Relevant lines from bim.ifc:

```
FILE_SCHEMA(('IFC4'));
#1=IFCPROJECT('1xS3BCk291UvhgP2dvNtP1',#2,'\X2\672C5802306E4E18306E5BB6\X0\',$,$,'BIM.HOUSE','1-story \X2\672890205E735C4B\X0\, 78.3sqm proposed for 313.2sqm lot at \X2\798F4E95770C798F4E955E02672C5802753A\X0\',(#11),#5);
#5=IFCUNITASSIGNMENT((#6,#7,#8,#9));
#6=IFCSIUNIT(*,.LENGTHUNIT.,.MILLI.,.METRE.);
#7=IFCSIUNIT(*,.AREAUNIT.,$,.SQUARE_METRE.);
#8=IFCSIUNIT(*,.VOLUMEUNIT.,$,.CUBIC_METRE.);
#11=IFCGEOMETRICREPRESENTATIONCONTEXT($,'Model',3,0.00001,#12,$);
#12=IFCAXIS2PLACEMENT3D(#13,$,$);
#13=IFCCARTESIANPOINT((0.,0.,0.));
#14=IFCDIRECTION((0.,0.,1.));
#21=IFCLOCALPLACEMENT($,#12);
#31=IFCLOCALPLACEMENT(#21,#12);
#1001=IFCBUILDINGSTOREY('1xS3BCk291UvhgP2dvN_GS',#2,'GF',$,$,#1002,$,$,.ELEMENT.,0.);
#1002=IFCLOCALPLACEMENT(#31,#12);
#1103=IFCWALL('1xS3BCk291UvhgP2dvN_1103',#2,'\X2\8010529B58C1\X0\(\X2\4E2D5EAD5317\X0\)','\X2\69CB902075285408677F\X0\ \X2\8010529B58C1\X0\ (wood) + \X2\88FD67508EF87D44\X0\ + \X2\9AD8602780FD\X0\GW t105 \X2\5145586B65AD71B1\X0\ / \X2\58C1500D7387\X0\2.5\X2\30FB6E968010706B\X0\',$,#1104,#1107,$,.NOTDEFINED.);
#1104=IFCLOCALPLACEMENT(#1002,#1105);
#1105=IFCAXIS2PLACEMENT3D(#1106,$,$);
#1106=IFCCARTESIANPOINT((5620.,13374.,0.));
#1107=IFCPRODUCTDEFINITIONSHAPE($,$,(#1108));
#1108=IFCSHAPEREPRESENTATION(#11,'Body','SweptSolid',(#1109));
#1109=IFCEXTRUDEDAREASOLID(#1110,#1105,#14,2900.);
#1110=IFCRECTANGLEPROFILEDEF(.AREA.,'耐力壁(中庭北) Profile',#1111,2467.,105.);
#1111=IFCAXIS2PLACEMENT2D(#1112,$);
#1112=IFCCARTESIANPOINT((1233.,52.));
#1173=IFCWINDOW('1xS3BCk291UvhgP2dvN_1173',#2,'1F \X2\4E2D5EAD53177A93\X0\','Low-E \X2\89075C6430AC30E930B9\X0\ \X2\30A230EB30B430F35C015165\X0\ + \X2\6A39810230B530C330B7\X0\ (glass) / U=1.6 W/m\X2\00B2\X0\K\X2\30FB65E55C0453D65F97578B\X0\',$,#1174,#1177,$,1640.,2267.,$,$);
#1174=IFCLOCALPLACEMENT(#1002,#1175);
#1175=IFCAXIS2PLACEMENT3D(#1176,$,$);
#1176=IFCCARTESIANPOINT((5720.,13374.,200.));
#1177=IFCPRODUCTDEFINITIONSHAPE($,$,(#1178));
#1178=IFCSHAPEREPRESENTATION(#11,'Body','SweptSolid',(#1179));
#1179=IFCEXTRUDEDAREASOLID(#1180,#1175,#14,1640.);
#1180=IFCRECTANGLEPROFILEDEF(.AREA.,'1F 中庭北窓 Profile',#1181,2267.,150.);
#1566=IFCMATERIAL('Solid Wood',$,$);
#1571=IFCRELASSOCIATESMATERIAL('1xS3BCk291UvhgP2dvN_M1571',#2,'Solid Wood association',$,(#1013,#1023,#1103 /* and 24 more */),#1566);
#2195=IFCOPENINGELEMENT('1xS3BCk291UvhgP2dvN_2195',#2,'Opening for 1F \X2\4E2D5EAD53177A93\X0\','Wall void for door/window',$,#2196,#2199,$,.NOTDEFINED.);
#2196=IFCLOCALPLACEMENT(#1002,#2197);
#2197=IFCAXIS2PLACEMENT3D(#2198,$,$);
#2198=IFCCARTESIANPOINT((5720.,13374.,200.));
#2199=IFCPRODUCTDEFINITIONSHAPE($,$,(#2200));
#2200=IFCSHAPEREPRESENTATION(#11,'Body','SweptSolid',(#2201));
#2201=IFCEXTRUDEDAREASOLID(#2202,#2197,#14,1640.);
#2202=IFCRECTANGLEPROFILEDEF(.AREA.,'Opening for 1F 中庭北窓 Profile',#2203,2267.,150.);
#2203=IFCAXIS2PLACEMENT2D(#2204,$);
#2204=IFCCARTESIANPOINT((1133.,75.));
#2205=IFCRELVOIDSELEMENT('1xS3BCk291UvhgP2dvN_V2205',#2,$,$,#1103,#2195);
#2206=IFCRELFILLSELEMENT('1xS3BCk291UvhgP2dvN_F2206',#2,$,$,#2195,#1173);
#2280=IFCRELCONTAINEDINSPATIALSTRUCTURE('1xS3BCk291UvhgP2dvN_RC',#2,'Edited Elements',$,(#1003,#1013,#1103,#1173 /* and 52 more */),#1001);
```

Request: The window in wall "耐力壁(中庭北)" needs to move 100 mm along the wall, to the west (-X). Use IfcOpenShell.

```python
import ifcopenshell
import ifcopenshell.api.geometry
import ifcopenshell.util.placement
import ifcopenshell.util.unit

model = ifcopenshell.open("bim.ifc")
unit_scale = ifcopenshell.util.unit.calculate_unit_scale(model)

window = model.by_guid("1xS3BCk291UvhgP2dvN_1173")
opening = window.FillsVoids[0].RelatingOpeningElement
wall = opening.VoidsElements[0].RelatingBuildingElement

wall_matrix = ifcopenshell.util.placement.get_local_placement(wall.ObjectPlacement)
shift = wall_matrix[:3, 0] * -0.1 / unit_scale
before = ifcopenshell.util.placement.get_local_placement(window.ObjectPlacement)[:3, 3].copy()

# The window is not placed relative to its opening, so move both.
for product in (opening, window):
    matrix = ifcopenshell.util.placement.get_local_placement(product.ObjectPlacement)
    matrix[:3, 3] += shift
    ifcopenshell.api.geometry.edit_object_placement(model, product=product, matrix=matrix, is_si=False)

after = ifcopenshell.util.placement.get_local_placement(window.ObjectPlacement)[:3, 3]
print("window moved by", (after - before).round(3) + 0.0)

model.write("bim_rev.ifc")
```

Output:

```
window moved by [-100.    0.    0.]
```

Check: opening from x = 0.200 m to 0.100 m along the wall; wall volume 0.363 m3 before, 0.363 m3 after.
